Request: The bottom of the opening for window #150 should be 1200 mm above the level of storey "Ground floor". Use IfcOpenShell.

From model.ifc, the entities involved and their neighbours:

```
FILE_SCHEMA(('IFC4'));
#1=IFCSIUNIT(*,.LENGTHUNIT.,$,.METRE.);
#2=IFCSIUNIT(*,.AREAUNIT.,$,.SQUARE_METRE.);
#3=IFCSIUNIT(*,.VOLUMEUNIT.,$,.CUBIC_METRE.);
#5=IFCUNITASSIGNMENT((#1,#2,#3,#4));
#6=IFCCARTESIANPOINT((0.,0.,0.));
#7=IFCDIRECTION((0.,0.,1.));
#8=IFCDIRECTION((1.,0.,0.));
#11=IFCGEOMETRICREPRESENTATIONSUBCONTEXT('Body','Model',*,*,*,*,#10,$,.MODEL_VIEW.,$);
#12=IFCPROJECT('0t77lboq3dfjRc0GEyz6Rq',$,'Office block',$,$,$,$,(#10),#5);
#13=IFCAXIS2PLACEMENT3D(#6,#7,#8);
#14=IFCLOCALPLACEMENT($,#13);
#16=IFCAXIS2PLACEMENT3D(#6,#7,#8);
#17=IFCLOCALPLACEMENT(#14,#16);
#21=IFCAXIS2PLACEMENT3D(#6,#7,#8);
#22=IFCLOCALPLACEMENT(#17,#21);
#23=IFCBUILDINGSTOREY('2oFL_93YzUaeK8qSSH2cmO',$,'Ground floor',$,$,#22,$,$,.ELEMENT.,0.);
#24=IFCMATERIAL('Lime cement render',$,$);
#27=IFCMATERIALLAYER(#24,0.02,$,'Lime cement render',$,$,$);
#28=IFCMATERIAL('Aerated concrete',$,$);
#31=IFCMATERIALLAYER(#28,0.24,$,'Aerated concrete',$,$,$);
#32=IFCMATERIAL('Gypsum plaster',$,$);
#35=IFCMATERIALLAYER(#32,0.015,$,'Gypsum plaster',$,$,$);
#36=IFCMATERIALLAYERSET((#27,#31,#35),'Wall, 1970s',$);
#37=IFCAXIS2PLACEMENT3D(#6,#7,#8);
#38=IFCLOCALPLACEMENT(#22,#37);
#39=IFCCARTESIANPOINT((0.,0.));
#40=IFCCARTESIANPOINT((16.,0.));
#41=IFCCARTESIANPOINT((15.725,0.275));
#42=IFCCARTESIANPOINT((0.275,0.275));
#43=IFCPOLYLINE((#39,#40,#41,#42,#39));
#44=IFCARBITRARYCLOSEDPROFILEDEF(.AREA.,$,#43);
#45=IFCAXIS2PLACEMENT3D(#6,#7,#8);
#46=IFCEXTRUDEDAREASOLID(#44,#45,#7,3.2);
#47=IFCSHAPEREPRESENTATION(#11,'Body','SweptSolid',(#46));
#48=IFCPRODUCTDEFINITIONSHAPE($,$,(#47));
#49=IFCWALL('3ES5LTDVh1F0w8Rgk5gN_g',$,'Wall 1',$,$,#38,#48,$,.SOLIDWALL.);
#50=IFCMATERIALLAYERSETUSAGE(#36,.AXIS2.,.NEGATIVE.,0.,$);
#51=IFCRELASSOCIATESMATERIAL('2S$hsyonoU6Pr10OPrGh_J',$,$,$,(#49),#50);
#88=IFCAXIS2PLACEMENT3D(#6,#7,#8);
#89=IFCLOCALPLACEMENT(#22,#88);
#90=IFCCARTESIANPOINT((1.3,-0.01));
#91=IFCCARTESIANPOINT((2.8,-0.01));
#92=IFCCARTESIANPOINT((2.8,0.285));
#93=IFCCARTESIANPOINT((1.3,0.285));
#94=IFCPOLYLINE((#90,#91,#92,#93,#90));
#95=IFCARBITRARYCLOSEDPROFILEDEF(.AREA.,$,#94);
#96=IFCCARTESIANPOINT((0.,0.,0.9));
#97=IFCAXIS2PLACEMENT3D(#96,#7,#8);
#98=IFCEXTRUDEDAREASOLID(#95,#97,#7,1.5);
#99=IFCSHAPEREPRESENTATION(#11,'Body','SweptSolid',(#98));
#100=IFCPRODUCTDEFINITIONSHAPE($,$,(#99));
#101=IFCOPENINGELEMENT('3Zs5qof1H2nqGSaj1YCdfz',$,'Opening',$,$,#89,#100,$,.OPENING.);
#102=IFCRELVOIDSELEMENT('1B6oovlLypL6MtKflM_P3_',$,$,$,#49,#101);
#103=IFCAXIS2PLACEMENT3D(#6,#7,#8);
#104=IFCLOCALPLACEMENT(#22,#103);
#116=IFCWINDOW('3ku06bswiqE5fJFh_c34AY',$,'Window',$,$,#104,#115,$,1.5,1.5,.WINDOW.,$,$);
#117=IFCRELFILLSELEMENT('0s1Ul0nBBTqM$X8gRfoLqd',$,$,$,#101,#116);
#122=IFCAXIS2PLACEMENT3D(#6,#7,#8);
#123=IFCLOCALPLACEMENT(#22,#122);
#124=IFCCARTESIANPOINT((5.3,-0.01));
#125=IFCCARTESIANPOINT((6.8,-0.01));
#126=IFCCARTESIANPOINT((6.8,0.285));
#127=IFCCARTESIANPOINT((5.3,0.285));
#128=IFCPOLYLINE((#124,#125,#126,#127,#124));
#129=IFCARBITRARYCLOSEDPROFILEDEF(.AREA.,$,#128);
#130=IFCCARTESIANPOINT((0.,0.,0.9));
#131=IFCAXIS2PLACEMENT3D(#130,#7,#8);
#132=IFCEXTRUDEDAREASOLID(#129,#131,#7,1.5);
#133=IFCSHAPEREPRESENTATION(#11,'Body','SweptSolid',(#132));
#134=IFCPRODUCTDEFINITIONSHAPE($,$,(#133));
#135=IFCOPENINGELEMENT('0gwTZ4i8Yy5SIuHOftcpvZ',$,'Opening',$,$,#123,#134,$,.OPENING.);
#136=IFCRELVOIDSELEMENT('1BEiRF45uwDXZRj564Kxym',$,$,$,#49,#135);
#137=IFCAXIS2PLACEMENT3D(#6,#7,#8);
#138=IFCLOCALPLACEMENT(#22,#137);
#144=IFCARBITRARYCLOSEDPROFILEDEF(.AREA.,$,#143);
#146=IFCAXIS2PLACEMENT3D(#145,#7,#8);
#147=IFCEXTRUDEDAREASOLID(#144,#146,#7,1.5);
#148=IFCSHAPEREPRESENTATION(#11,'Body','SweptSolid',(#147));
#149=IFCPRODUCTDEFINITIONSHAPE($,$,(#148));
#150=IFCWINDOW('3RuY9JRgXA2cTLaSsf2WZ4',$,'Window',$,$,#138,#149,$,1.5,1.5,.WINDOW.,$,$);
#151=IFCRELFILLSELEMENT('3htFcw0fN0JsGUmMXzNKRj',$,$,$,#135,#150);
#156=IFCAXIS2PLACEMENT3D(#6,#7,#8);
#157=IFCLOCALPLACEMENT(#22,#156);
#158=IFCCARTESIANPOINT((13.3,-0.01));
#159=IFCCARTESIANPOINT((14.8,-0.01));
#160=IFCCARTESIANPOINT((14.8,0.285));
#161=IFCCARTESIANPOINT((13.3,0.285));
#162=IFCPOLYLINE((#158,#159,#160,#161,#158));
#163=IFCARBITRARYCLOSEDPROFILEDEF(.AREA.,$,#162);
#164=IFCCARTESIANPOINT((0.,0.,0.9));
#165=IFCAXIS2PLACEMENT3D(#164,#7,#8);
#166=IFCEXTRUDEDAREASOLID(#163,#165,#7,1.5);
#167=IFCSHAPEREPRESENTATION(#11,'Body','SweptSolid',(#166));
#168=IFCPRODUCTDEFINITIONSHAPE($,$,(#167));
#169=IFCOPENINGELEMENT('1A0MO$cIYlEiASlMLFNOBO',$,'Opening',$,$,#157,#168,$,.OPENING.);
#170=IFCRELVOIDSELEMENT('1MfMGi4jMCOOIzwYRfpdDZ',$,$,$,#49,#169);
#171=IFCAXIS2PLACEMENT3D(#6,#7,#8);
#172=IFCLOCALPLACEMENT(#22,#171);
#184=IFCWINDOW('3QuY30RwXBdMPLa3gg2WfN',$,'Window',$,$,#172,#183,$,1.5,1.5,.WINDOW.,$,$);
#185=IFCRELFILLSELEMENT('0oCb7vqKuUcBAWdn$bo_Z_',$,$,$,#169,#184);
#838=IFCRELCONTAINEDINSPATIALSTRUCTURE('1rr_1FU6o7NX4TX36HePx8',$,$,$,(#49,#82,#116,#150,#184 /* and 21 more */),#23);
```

```python
import numpy as np
import ifcopenshell
import ifcopenshell.api.geometry
import ifcopenshell.geom
import ifcopenshell.util.element
import ifcopenshell.util.placement
import ifcopenshell.util.shape
import ifcopenshell.util.unit

model = ifcopenshell.open("model.ifc")
unit_scale = ifcopenshell.util.unit.calculate_unit_scale(model)

window = model.by_guid("3RuY9JRgXA2cTLaSsf2WZ4")
opening = window.FillsVoids[0].RelatingOpeningElement
storey = ifcopenshell.util.element.get_container(window, ifc_class="IfcBuildingStorey")
level = ifcopenshell.util.placement.get_local_placement(storey.ObjectPlacement)[2, 3]

# The opening's origin need not be at the sill, so measure its lowest point.
shape = ifcopenshell.geom.create_shape(ifcopenshell.geom.settings(), opening)
bottom = ifcopenshell.util.shape.get_shape_bottom_elevation(shape, shape.geometry) / unit_scale
dz = level + 1.2 / unit_scale - bottom

shift = np.array([0.0, 0.0, dz])
# The window is not placed relative to its opening, so move both.
for product in (opening, window):
    matrix = ifcopenshell.util.placement.get_local_placement(product.ObjectPlacement)
    matrix[:3, 3] += shift
    ifcopenshell.api.geometry.edit_object_placement(model, product=product, matrix=matrix, is_si=False)

print(f"moved by {dz * unit_scale:+.3f} m")

model.write("model-out.ifc")
```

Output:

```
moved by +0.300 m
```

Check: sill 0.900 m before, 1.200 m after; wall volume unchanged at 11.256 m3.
